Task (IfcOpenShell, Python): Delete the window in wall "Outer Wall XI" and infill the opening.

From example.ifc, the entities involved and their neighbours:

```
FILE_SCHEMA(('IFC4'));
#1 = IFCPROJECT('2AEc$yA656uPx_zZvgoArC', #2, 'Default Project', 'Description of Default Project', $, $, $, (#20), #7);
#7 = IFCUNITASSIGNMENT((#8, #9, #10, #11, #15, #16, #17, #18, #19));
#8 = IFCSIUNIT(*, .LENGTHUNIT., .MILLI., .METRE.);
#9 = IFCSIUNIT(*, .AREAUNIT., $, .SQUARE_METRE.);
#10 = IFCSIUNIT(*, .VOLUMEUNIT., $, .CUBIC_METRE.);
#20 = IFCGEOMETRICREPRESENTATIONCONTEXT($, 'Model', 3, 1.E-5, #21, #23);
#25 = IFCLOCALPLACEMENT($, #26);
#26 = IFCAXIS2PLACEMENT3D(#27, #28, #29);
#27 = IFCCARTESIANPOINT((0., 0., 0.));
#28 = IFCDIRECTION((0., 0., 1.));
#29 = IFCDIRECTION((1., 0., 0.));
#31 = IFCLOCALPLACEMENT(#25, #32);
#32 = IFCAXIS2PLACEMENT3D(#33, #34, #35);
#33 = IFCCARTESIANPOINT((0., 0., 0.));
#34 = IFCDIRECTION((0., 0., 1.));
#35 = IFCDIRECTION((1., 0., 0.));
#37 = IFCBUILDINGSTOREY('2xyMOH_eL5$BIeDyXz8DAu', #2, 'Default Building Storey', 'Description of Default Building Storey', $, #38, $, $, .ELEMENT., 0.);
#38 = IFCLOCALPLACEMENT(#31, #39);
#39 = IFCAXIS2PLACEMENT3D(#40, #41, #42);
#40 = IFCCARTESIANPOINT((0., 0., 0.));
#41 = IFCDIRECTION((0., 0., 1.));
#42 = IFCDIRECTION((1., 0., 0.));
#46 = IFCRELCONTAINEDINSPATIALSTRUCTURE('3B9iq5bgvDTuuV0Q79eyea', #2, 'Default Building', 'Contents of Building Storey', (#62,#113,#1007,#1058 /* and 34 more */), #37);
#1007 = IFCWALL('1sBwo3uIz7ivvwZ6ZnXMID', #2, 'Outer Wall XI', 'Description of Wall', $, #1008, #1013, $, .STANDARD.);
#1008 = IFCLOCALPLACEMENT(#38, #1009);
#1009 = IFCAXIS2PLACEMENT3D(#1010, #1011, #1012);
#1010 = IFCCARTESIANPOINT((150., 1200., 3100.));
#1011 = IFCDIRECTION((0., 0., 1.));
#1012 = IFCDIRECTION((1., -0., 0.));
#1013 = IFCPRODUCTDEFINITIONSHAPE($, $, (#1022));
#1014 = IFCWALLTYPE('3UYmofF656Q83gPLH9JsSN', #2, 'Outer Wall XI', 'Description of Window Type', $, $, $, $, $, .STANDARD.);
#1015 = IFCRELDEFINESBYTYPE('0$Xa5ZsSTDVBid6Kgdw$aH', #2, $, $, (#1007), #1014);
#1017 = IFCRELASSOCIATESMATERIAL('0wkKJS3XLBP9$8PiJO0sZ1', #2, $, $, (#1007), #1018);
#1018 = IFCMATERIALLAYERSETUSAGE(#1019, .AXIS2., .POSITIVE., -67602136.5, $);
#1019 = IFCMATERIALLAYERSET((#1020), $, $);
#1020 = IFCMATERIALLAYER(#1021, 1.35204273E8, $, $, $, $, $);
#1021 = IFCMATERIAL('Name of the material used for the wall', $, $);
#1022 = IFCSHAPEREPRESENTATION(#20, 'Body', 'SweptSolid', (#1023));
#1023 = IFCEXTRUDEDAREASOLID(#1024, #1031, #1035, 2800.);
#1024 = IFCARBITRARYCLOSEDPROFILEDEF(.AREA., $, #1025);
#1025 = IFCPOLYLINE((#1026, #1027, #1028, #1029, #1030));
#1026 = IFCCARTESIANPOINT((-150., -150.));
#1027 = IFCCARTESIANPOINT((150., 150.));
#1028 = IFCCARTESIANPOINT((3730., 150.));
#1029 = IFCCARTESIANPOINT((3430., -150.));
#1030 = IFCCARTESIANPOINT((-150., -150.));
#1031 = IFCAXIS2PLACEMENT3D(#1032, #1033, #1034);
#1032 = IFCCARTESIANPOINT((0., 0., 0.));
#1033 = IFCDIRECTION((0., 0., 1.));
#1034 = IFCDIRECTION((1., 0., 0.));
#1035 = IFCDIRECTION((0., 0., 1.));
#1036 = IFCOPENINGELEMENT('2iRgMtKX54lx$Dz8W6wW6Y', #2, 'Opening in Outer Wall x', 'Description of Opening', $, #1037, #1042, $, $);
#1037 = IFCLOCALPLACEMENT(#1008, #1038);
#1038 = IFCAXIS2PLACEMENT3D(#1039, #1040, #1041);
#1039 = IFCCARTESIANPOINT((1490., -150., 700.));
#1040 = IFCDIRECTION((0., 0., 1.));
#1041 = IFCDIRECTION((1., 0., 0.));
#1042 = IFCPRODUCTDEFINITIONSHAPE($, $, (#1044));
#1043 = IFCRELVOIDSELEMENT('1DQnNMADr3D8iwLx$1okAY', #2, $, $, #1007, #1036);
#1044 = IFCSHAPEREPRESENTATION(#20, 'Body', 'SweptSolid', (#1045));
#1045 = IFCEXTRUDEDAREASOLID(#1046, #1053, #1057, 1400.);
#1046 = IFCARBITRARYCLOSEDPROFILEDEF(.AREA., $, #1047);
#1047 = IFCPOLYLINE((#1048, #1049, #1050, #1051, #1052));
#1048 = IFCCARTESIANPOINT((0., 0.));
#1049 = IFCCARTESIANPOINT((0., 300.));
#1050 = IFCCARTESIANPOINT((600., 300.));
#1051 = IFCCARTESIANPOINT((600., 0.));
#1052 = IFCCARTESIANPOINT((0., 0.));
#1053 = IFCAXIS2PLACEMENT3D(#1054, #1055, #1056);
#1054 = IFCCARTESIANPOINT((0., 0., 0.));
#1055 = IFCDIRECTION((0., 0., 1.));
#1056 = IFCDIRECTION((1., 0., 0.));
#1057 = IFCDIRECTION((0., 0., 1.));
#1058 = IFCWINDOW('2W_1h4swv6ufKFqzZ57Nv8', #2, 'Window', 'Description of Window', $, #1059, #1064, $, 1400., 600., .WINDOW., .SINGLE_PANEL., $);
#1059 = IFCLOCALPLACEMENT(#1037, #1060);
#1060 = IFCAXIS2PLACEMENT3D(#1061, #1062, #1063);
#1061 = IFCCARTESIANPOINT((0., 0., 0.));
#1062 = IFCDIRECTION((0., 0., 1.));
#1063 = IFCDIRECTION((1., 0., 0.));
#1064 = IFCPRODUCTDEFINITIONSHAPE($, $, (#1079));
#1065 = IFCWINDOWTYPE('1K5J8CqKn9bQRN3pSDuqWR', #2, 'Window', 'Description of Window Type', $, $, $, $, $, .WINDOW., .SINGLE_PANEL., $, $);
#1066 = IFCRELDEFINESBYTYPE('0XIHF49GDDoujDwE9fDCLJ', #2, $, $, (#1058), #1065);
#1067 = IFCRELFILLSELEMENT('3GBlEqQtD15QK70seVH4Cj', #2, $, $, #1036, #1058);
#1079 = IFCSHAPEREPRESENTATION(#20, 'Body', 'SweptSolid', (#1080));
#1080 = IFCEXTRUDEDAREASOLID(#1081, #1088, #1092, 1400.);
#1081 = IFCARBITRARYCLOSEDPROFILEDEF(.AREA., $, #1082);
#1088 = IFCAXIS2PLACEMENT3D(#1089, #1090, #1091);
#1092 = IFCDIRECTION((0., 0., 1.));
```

```python
import ifcopenshell
import ifcopenshell.api.feature
import ifcopenshell.api.root
import ifcopenshell.geom
import ifcopenshell.util.shape

model = ifcopenshell.open("example.ifc")
settings = ifcopenshell.geom.settings()


def volume(element):
    """Net volume in cubic metres, openings subtracted."""
    shape = ifcopenshell.geom.create_shape(settings, element)
    return ifcopenshell.util.shape.get_volume(shape.geometry)


window = model.by_guid("2W_1h4swv6ufKFqzZ57Nv8")
opening = window.FillsVoids[0].RelatingOpeningElement
wall = opening.VoidsElements[0].RelatingBuildingElement
before = volume(wall)

ifcopenshell.api.root.remove_product(model, product=window)
ifcopenshell.api.feature.remove_feature(model, feature=opening)

after = volume(wall)

print(f"wall volume {before:.3f} -> {after:.3f} m3")

model.write("example_v2.ifc")
```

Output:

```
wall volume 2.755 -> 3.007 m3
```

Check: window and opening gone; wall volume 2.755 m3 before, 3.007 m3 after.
